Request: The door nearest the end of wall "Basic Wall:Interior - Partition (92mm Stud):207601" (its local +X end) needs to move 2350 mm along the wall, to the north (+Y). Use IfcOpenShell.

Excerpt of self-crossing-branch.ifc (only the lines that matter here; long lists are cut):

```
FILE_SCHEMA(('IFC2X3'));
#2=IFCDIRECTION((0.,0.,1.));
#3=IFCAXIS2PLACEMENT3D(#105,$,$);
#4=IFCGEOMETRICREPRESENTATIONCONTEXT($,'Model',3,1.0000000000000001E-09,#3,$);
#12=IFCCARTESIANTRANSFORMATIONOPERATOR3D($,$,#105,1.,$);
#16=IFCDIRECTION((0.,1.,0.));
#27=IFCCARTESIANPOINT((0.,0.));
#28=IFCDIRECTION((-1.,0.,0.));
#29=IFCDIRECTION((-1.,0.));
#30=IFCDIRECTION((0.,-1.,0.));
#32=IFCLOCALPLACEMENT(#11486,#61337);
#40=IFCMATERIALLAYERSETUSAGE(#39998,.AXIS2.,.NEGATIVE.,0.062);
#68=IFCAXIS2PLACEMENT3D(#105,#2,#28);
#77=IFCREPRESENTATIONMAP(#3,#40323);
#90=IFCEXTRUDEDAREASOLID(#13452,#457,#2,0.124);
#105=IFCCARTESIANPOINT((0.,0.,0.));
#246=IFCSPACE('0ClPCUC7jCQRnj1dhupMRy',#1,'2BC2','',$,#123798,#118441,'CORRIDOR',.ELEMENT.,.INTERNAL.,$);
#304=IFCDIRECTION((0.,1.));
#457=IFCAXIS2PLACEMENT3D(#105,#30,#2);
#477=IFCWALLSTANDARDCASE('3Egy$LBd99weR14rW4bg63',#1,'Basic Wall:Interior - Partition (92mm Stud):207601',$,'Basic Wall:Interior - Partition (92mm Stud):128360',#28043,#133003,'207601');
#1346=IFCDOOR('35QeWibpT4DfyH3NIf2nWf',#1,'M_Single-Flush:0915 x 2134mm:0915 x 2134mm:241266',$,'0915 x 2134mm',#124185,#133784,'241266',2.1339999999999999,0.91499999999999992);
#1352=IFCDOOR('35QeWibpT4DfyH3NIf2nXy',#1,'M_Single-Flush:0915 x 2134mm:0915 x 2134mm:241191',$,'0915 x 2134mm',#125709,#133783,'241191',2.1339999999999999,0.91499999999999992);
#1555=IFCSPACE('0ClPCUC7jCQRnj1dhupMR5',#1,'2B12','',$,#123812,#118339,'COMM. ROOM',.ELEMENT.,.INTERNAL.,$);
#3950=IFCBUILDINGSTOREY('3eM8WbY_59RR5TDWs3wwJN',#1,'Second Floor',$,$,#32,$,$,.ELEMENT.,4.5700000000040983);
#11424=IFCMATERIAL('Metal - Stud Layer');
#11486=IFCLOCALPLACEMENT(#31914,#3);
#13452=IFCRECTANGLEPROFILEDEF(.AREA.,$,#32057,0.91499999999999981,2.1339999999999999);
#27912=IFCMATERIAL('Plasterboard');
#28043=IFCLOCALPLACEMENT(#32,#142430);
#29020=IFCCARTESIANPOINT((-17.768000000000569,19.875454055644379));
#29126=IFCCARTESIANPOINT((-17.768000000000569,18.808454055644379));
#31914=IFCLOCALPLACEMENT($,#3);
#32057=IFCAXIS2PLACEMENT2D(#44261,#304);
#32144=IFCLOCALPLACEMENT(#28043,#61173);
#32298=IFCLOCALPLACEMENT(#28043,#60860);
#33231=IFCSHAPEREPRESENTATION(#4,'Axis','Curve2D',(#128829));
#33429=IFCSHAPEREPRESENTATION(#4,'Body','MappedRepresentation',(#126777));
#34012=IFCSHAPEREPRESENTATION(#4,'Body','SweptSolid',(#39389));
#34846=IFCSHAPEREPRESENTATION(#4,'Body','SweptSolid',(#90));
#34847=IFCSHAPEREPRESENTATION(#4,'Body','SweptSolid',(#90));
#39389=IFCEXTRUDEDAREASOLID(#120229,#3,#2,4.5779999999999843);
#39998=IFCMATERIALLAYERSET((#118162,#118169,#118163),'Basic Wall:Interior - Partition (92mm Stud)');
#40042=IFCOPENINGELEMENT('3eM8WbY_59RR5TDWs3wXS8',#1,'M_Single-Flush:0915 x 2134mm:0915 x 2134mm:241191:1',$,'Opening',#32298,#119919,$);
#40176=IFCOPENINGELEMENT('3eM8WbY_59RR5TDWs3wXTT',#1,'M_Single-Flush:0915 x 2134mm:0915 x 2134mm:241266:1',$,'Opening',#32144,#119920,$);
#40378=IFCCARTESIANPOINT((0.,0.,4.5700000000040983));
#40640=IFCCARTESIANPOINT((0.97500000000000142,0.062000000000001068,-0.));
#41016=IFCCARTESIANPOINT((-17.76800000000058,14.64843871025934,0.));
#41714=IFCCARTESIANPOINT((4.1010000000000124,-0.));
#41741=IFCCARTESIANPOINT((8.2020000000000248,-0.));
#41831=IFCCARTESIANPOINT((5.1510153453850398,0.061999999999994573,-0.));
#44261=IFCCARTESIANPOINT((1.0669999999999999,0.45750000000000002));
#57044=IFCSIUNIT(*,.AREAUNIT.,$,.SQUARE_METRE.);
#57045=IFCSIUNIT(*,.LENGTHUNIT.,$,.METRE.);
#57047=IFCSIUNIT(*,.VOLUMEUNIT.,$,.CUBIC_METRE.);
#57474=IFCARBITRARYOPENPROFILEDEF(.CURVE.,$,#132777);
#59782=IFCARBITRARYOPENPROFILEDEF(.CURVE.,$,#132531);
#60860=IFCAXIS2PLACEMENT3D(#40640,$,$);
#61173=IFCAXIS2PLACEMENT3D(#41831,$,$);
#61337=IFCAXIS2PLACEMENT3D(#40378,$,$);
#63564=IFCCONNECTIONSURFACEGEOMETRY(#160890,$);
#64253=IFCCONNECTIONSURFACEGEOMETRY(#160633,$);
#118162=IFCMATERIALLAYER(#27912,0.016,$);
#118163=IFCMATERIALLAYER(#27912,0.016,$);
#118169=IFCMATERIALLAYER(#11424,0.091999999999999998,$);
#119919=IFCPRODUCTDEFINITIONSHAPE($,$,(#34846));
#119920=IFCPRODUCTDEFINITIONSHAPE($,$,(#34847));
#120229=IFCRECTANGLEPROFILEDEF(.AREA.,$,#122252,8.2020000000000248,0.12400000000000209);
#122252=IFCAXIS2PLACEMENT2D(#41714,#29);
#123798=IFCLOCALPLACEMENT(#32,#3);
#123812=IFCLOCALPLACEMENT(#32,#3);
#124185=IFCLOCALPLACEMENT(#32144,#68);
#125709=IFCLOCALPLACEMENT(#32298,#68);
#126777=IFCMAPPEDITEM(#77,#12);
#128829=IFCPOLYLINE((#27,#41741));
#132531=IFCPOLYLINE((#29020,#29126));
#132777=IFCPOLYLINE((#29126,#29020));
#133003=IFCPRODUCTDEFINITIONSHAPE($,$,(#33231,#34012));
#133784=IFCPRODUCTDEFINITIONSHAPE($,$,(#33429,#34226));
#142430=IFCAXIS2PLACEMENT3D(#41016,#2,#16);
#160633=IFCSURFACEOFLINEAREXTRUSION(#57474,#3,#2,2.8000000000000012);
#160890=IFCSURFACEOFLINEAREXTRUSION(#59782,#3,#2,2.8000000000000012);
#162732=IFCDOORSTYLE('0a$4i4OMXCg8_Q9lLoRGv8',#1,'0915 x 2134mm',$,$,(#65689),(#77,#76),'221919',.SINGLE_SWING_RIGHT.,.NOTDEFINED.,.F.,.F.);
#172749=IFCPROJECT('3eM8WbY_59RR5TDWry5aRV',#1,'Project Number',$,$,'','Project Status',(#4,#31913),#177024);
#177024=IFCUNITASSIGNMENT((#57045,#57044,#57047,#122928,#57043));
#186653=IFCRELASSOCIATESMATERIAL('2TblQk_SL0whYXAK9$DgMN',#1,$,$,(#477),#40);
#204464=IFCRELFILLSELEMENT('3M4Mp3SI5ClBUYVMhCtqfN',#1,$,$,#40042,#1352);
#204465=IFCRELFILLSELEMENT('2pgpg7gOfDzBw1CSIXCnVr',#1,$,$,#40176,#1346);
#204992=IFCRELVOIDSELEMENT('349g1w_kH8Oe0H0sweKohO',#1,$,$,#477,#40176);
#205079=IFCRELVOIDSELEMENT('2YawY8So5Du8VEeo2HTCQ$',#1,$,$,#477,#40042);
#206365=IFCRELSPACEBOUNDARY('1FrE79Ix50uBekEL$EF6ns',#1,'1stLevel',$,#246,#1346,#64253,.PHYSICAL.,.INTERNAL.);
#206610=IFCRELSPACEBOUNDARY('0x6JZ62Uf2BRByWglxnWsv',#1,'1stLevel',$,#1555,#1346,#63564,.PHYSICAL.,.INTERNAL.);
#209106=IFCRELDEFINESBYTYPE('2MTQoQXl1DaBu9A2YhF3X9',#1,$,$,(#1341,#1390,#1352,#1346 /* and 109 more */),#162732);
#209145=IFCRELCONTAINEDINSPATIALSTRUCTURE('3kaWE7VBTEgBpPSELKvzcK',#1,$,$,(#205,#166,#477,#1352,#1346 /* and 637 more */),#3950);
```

```python
import numpy as np
import ifcopenshell
import ifcopenshell.api.geometry
import ifcopenshell.util.placement

model = ifcopenshell.open("self-crossing-branch.ifc")

door = model.by_guid("35QeWibpT4DfyH3NIf2nWf")
opening = door.FillsVoids[0].RelatingOpeningElement
wall = opening.VoidsElements[0].RelatingBuildingElement

wall_matrix = ifcopenshell.util.placement.get_local_placement(wall.ObjectPlacement)
shift = wall_matrix[:3, 0] * 2.35
before = ifcopenshell.util.placement.get_local_placement(door.ObjectPlacement)[:3, 3].copy()

# The door is placed relative to its opening, so it follows when the opening moves.
matrix = ifcopenshell.util.placement.get_local_placement(opening.ObjectPlacement)
matrix[:3, 3] += shift
ifcopenshell.api.geometry.edit_object_placement(
    model, product=opening, matrix=matrix, is_si=False, should_transform_children=True
)

# Space boundary surfaces are stored in each space's coordinates; move them too.
for rel in door.ProvidesBoundaries:
    if not rel.ConnectionGeometry:
        continue
    surface = rel.ConnectionGeometry.SurfaceOnRelatingElement
    space_matrix = ifcopenshell.util.placement.get_local_placement(rel.RelatingSpace.ObjectPlacement)
    point = np.array(surface.Position.Location.Coordinates) + space_matrix[:3, :3].T @ shift
    surface.Position = model.createIfcAxis2Placement3D(
        model.createIfcCartesianPoint(point.tolist()), surface.Position.Axis, surface.Position.RefDirection
    )

after = ifcopenshell.util.placement.get_local_placement(door.ObjectPlacement)[:3, 3]
print("door moved by", (after - before).round(3) + 0.0)

model.write("self-crossing-branch-out.ifc")
```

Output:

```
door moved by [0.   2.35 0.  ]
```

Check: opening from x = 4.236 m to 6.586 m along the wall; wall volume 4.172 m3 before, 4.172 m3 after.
